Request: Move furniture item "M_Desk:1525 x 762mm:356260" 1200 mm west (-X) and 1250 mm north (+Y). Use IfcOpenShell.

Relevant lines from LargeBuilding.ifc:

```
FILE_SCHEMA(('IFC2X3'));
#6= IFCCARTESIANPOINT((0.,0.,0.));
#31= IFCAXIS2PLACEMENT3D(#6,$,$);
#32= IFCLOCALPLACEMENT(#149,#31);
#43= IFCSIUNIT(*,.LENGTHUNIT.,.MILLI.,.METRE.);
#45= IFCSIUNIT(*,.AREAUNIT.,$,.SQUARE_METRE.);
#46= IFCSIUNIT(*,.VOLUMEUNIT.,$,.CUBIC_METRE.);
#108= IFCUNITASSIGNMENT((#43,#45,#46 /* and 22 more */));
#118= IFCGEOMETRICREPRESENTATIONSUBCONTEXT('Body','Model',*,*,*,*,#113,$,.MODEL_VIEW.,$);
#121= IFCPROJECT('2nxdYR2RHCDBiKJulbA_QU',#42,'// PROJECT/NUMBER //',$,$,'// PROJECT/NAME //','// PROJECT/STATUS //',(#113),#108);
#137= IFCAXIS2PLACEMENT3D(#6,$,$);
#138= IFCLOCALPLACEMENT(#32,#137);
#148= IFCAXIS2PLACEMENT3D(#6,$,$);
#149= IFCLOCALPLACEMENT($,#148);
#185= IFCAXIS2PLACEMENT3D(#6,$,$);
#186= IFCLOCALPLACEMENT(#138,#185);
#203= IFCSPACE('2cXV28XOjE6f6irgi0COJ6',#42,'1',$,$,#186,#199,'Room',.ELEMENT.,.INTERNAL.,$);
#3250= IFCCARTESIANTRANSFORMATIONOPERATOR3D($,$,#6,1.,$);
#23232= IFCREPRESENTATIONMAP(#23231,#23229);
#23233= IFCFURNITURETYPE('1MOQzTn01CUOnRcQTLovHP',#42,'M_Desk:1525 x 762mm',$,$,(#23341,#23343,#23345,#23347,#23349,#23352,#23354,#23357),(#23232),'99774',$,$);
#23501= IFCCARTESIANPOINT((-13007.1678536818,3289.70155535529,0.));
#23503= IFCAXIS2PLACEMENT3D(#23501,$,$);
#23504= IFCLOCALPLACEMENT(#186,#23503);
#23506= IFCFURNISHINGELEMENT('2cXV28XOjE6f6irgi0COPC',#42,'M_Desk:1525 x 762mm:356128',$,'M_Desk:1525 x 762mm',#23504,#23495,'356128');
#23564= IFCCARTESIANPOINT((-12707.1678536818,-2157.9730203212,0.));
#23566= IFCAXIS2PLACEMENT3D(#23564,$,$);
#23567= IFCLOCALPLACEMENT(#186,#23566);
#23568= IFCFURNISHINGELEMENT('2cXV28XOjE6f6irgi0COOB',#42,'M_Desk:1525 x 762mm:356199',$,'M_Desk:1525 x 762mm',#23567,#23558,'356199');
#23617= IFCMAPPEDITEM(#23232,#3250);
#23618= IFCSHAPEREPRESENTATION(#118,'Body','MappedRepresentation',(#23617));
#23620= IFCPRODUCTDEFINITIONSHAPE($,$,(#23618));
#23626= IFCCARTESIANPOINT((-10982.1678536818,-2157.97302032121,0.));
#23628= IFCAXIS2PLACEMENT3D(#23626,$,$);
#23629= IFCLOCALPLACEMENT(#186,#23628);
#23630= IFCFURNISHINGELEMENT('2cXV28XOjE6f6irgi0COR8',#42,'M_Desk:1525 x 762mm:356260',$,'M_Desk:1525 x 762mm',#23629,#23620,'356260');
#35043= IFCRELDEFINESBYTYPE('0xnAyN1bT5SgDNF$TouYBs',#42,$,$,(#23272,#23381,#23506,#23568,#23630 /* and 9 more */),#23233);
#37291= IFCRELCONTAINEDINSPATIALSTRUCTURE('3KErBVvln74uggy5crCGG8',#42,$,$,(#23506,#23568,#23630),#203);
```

```python
import ifcopenshell
import ifcopenshell.api.geometry
import ifcopenshell.util.placement
import ifcopenshell.util.unit

model = ifcopenshell.open("LargeBuilding.ifc")
unit_scale = ifcopenshell.util.unit.calculate_unit_scale(model)

item = model.by_id(23630)
matrix = ifcopenshell.util.placement.get_local_placement(item.ObjectPlacement)
matrix[0, 3] -= 1.2 / unit_scale
matrix[1, 3] += 1.25 / unit_scale
ifcopenshell.api.geometry.edit_object_placement(model, product=item, matrix=matrix, is_si=False)

print(ifcopenshell.util.placement.get_local_placement(item.ObjectPlacement).round(3) + 0.0)

model.write("LargeBuilding_edited.ifc")
```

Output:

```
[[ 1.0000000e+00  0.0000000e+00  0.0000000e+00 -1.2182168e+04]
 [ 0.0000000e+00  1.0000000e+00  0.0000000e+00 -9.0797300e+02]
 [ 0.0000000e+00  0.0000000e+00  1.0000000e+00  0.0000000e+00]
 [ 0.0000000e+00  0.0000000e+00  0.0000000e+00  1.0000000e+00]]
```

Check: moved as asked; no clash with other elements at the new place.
